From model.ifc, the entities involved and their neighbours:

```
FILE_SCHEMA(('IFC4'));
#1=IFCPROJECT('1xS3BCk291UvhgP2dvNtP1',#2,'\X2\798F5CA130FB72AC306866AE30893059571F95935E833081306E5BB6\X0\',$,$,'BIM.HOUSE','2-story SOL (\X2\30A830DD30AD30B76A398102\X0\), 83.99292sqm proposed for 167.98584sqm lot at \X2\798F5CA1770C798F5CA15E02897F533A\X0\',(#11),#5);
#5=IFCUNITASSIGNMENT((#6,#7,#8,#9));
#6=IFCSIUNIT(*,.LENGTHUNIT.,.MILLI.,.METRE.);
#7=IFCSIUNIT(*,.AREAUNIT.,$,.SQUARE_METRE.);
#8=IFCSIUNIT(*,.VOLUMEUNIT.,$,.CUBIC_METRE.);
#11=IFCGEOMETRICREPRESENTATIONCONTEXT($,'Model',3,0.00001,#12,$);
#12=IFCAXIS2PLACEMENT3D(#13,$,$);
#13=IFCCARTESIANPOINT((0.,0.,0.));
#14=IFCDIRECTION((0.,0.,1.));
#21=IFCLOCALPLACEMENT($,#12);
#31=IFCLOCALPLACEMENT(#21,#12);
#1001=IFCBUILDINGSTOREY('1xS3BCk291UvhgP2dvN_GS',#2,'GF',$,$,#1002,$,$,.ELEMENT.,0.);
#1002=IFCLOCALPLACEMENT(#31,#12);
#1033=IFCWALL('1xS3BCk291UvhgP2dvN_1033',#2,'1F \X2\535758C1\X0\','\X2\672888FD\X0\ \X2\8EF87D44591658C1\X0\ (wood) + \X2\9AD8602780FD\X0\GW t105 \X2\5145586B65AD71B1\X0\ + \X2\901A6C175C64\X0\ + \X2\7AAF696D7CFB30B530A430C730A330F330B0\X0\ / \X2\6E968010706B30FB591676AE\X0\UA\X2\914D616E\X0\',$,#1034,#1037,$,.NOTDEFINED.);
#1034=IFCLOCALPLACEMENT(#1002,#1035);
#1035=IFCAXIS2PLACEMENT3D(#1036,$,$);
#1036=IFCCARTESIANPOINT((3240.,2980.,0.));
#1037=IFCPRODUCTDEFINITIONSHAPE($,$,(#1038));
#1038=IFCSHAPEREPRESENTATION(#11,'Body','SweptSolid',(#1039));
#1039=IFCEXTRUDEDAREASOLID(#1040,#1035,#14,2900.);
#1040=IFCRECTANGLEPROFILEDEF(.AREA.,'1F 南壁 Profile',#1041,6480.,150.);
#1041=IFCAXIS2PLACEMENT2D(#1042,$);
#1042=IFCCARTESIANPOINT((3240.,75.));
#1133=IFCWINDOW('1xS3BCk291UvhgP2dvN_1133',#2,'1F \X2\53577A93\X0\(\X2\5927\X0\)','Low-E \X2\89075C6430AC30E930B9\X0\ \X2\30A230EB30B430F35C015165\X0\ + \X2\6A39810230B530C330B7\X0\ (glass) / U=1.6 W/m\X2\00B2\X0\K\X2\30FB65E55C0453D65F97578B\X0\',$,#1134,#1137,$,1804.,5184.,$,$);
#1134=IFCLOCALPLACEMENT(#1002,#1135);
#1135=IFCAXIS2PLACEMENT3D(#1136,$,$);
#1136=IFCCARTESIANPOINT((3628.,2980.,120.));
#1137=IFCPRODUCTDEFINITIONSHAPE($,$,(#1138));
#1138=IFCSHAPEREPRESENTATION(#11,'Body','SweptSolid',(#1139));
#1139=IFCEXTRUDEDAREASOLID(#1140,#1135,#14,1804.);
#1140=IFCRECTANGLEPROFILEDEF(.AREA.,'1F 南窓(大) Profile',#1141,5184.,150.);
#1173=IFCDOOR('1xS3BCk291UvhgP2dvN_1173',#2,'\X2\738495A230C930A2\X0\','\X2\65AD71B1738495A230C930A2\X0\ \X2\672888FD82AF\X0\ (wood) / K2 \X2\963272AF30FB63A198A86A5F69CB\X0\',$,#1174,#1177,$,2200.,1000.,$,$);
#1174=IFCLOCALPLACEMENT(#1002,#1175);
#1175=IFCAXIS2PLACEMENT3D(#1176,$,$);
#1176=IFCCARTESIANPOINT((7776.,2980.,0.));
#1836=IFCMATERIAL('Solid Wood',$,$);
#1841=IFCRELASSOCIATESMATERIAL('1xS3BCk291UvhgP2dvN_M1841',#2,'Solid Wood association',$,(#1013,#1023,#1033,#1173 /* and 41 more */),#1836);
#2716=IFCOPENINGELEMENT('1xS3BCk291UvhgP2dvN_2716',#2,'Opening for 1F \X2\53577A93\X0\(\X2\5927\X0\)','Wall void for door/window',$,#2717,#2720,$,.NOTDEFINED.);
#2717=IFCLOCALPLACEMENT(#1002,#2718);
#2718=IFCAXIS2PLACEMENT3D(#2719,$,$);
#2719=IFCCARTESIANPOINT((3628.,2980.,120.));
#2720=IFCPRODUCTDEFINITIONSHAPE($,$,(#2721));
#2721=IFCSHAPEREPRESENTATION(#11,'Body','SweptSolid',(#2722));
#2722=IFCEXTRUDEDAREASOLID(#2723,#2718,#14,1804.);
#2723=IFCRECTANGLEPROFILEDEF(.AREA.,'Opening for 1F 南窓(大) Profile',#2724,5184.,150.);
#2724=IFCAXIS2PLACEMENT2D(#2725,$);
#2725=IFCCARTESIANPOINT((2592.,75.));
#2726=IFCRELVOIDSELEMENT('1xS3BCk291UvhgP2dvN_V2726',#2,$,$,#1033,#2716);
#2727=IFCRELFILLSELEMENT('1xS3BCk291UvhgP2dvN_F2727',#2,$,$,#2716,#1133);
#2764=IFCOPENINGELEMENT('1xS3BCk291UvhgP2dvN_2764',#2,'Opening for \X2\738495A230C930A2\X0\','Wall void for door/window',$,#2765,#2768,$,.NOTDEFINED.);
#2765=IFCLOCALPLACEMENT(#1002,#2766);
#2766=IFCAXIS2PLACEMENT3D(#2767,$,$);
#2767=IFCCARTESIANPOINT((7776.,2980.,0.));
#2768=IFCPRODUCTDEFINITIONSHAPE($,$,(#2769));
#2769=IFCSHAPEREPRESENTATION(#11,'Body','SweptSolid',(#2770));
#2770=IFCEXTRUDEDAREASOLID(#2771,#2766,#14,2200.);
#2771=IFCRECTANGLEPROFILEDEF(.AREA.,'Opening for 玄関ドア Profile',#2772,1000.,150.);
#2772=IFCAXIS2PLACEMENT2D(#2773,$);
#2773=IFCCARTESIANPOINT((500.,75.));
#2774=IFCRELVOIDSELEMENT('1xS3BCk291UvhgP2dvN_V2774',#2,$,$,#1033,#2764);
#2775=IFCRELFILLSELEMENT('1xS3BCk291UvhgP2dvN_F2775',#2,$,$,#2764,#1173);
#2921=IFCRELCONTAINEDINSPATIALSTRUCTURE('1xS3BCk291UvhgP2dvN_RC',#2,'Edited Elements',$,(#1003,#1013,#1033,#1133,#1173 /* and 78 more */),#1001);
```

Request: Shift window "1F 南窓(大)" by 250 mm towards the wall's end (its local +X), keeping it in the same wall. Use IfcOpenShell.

```python
import ifcopenshell
import ifcopenshell.api.geometry
import ifcopenshell.util.placement
import ifcopenshell.util.unit

model = ifcopenshell.open("model.ifc")
unit_scale = ifcopenshell.util.unit.calculate_unit_scale(model)

window = model.by_guid("1xS3BCk291UvhgP2dvN_1133")
opening = window.FillsVoids[0].RelatingOpeningElement
wall = opening.VoidsElements[0].RelatingBuildingElement

wall_matrix = ifcopenshell.util.placement.get_local_placement(wall.ObjectPlacement)
shift = wall_matrix[:3, 0] * 0.25 / unit_scale
before = ifcopenshell.util.placement.get_local_placement(window.ObjectPlacement)[:3, 3].copy()

# The window is not placed relative to its opening, so move both.
for product in (opening, window):
    matrix = ifcopenshell.util.placement.get_local_placement(product.ObjectPlacement)
    matrix[:3, 3] += shift
    ifcopenshell.api.geometry.edit_object_placement(model, product=product, matrix=matrix, is_si=False)

after = ifcopenshell.util.placement.get_local_placement(window.ObjectPlacement)[:3, 3]
print("window moved by", (after - before).round(3) + 0.0)

model.write("model_rev.ifc")
```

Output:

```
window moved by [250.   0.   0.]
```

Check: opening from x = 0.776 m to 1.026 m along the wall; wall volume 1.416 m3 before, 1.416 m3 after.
